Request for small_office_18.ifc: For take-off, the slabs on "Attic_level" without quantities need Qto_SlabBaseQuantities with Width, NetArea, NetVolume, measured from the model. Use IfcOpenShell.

First a look at what the model holds.

```python
import ifcopenshell
import ifcopenshell.util.element
import ifcopenshell.util.unit

model = ifcopenshell.open("small_office_18.ifc")
print(model.schema)
for unit_type in ("LENGTHUNIT", "AREAUNIT", "VOLUMEUNIT"):
    print(unit_type, ifcopenshell.util.unit.calculate_unit_scale(model, unit_type))
storey = next(s for s in model.by_type("IfcBuildingStorey") if s.Name == "Attic_level")
slabs = [e for e in ifcopenshell.util.element.get_decomposition(storey) if e.is_a("IfcSlab")]
for e in sorted(slabs, key=lambda e: e.id()):
    print(e.id(), e.is_a(), e.Name, list(ifcopenshell.util.element.get_psets(e, qtos_only=True)), sep=" | ")
```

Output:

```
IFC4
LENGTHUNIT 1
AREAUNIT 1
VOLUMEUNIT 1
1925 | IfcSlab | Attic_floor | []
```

```python
import ifcopenshell
import ifcopenshell.api.pset
import ifcopenshell.geom
import ifcopenshell.util.element
import ifcopenshell.util.shape
import ifcopenshell.util.unit

model = ifcopenshell.open("small_office_18.ifc")
unit_scale = ifcopenshell.util.unit.calculate_unit_scale(model)
area_scale = ifcopenshell.util.unit.calculate_unit_scale(model, "AREAUNIT")
volume_scale = ifcopenshell.util.unit.calculate_unit_scale(model, "VOLUMEUNIT")
settings = ifcopenshell.geom.settings()

storey = next(s for s in model.by_type("IfcBuildingStorey") if s.Name == "Attic_level")
slabs = [e for e in ifcopenshell.util.element.get_decomposition(storey) if e.is_a("IfcSlab")]

for e in sorted(slabs, key=lambda e: e.id()):
    if ifcopenshell.util.element.get_psets(e, qtos_only=True, should_inherit=False):
        continue
    # Geometry comes back in metres, in the element's own axes.
    shape = ifcopenshell.geom.create_shape(settings, e)
    values = {
        "Width": ifcopenshell.util.shape.get_z(shape.geometry) / unit_scale,
        "NetArea": ifcopenshell.util.shape.get_footprint_area(shape.geometry) / area_scale,
        "NetVolume": ifcopenshell.util.shape.get_volume(shape.geometry) / volume_scale,
    }
    qto = ifcopenshell.api.pset.add_qto(model, product=e, name="Qto_SlabBaseQuantities")
    ifcopenshell.api.pset.edit_qto(model, qto=qto, properties=values)
    print(e.id(), {k: round(v, 3) for k, v in values.items()})

model.write("small_office_18-out.ifc")
```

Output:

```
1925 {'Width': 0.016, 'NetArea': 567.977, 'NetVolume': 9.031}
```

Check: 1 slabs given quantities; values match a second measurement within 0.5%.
